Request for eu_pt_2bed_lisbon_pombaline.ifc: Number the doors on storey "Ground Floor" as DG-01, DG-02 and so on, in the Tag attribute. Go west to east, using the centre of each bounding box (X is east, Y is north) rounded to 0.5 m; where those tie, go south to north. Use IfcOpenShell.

First a look at what the model holds.

```python
import ifcopenshell
import ifcopenshell.util.element
import ifcopenshell.util.placement

model = ifcopenshell.open("eu_pt_2bed_lisbon_pombaline.ifc")
print(model.schema)
storey = next(s for s in model.by_type("IfcBuildingStorey") if s.Name == "Ground Floor")
doors = [e for e in ifcopenshell.util.element.get_decomposition(storey) if e.is_a("IfcDoor")]
for e in sorted(doors, key=lambda e: e.id()):
    origin = ifcopenshell.util.placement.get_local_placement(e.ObjectPlacement)[:3, 3]
    print(e.id(), e.Tag, e.Name, origin.round(2) + 0.0, sep=" | ")
```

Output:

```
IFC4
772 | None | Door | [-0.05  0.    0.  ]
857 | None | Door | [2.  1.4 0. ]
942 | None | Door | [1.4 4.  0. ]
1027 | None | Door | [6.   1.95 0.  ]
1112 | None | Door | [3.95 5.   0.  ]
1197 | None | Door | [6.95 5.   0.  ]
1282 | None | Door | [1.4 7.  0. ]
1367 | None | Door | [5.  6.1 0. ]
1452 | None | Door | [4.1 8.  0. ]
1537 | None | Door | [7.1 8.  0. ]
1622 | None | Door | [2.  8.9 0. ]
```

```python
import ifcopenshell
import ifcopenshell.geom
import ifcopenshell.util.element
import ifcopenshell.util.shape

model = ifcopenshell.open("eu_pt_2bed_lisbon_pombaline.ifc")
settings = ifcopenshell.geom.settings()
settings.set("use-world-coords", True)


def centre(element):
    shape = ifcopenshell.geom.create_shape(settings, element)
    return ifcopenshell.util.shape.get_bbox_centroid(shape.geometry)


storey = next(s for s in model.by_type("IfcBuildingStorey") if s.Name == "Ground Floor")
doors = [e for e in ifcopenshell.util.element.get_decomposition(storey) if e.is_a("IfcDoor")]

# Insertion points can sit at a corner or the storey origin, so sort by the geometry (in metres).
centres = {e: centre(e) for e in doors}
doors.sort(key=lambda e: (round(centres[e][0] / 0.5), centres[e][1]))

for i, e in enumerate(doors, start=1):
    number = f"DG-{i:02d}"
    e.Tag = number
    print(e.id(), number)

model.write("eu_pt_2bed_lisbon_pombaline_rev.ifc")
```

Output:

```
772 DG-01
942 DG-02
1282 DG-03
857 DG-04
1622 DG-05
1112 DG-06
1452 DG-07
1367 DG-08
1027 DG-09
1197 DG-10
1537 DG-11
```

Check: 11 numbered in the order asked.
